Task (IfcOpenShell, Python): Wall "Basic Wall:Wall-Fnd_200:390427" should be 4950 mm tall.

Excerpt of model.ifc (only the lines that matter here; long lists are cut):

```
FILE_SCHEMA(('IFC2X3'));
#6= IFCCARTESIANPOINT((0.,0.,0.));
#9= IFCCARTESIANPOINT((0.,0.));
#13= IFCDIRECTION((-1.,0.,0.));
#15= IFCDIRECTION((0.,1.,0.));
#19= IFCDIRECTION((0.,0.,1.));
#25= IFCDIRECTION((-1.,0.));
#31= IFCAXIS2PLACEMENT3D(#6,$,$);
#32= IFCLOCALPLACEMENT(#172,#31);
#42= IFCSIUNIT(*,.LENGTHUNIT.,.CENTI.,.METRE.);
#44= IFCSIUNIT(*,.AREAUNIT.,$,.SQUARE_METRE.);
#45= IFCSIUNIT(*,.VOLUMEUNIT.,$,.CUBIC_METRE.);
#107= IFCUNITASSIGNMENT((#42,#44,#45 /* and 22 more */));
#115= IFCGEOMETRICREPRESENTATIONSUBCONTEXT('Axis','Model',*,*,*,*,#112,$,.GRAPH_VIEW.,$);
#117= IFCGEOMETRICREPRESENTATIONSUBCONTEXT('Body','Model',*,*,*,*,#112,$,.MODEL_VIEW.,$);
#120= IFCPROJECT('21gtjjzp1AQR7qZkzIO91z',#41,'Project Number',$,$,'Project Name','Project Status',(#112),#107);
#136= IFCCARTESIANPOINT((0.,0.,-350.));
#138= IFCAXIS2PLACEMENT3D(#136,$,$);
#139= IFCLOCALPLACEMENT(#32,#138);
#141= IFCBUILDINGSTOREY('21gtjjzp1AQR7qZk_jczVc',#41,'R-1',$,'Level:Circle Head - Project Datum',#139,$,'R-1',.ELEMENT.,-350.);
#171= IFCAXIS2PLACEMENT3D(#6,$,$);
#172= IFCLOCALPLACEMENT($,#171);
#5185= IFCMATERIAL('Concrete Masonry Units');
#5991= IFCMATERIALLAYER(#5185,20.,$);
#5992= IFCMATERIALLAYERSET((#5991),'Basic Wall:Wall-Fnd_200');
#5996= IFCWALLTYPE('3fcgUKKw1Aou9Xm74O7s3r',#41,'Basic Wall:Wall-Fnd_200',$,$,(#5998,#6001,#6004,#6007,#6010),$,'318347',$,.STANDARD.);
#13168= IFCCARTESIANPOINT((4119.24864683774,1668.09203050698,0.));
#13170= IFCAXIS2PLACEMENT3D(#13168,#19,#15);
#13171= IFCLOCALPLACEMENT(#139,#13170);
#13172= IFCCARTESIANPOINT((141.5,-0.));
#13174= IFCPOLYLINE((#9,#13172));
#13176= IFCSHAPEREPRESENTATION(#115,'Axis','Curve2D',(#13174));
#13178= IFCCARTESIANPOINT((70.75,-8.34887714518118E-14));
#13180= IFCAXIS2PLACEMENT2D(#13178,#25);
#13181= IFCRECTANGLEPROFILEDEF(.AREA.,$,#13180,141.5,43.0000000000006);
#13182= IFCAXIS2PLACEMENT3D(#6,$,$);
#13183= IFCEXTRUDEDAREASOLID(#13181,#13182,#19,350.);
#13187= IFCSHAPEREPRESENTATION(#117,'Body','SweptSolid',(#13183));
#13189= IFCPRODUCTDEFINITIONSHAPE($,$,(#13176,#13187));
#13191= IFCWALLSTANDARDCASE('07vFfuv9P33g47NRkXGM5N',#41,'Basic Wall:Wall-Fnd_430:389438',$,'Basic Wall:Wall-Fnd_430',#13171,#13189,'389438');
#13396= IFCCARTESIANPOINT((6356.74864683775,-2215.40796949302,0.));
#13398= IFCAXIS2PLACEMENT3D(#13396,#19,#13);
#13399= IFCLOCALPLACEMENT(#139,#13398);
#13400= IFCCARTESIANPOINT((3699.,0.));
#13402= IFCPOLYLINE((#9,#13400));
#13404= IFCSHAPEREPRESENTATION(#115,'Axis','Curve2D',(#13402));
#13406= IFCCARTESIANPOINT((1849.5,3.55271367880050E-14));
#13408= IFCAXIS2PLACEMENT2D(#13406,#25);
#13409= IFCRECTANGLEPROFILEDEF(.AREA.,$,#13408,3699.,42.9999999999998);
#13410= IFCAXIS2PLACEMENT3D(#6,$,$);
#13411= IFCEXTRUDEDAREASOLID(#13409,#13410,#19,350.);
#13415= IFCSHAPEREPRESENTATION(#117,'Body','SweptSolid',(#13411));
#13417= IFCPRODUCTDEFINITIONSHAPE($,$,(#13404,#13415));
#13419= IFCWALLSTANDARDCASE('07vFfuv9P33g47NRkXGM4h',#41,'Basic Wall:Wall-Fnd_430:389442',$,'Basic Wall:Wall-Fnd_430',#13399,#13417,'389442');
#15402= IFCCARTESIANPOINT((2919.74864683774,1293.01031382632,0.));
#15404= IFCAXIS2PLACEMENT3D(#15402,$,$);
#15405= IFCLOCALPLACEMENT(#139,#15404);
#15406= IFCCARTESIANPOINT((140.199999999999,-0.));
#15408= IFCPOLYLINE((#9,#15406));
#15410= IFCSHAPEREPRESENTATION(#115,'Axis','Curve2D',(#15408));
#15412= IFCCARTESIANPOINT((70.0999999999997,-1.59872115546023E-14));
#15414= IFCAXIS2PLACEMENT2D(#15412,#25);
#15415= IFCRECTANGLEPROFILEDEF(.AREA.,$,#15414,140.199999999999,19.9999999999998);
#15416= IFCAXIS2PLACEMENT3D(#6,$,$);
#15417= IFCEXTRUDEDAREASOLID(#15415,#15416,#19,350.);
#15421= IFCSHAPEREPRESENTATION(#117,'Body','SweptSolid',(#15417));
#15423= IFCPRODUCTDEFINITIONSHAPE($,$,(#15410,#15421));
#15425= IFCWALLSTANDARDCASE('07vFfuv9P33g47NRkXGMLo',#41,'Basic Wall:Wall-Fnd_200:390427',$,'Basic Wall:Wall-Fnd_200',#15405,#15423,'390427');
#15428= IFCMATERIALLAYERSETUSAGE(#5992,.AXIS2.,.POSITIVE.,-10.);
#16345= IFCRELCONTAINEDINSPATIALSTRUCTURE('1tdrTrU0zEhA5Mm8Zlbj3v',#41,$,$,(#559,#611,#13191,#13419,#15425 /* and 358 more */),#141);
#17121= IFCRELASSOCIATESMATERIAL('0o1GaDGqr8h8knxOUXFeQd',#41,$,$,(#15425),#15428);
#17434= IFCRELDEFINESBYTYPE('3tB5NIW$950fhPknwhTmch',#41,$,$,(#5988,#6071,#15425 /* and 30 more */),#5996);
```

```python
import ifcopenshell
import ifcopenshell.geom
import ifcopenshell.util.representation
import ifcopenshell.util.shape
import ifcopenshell.util.unit

model = ifcopenshell.open("model.ifc")
unit_scale = ifcopenshell.util.unit.calculate_unit_scale(model)
settings = ifcopenshell.geom.settings()


def volume(element):
    """Net volume in cubic metres, openings subtracted."""
    shape = ifcopenshell.geom.create_shape(settings, element)
    return ifcopenshell.util.shape.get_volume(shape.geometry)


wall = model.by_guid("07vFfuv9P33g47NRkXGMLo")
before = volume(wall)

body = ifcopenshell.util.representation.get_representation(wall, "Model", "Body")
solid = body.Items[0]
old_height = solid.Depth
solid.Depth = 4.95 / unit_scale
after = volume(wall)

print(f"height {old_height:g} -> {solid.Depth:g}, volume {before:.3f} -> {after:.3f} m3")

model.write("model_v2.ifc")
```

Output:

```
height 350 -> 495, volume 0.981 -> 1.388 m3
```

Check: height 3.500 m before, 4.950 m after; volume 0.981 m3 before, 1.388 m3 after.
